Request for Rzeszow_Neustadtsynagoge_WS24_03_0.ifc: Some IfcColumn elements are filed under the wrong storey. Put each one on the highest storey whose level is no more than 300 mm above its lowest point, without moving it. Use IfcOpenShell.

First a look at what the model holds.

```python
import ifcopenshell
import ifcopenshell.util.element
import ifcopenshell.util.placement

model = ifcopenshell.open("Rzeszow_Neustadtsynagoge_WS24_03_0.ifc")
print(model.schema)
for storey in model.by_type("IfcBuildingStorey"):
    level = ifcopenshell.util.placement.get_storey_elevation(storey)
    count = sum(e.is_a("IfcColumn") for e in ifcopenshell.util.element.get_contained(storey))
    print(storey.id(), storey.Name, round(level, 3), count, sep=" | ")
```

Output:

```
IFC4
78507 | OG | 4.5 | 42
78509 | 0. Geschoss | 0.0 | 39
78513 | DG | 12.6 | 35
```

```python
import ifcopenshell
import ifcopenshell.api.spatial
import ifcopenshell.geom
import ifcopenshell.util.element
import ifcopenshell.util.placement
import ifcopenshell.util.shape
import ifcopenshell.util.unit

model = ifcopenshell.open("Rzeszow_Neustadtsynagoge_WS24_03_0.ifc")
unit_scale = ifcopenshell.util.unit.calculate_unit_scale(model)
settings = ifcopenshell.geom.settings()

levels = sorted(
    ((ifcopenshell.util.placement.get_storey_elevation(s) * unit_scale, s) for s in model.by_type("IfcBuildingStorey")),
    key=lambda pair: pair[0],
)

for e in model.by_type("IfcColumn"):
    current = e.ContainedInStructure[0].RelatingStructure if e.ContainedInStructure else None
    if current is None or not current.is_a("IfcBuildingStorey"):
        continue
    shape = ifcopenshell.geom.create_shape(settings, e)
    bottom = ifcopenshell.util.shape.get_shape_bottom_elevation(shape, shape.geometry)
    below = [s for level, s in levels if level <= bottom + 0.3]
    storey = below[-1] if below else levels[0][1]
    if storey != current:
        # assign_container keeps the world position.
        ifcopenshell.api.spatial.assign_container(model, products=[e], relating_structure=storey)
        print(e.id(), current.Name, "->", storey.Name)

model.write("Rzeszow_Neustadtsynagoge_WS24_03_0_rev.ifc")
```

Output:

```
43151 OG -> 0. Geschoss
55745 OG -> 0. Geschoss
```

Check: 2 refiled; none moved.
